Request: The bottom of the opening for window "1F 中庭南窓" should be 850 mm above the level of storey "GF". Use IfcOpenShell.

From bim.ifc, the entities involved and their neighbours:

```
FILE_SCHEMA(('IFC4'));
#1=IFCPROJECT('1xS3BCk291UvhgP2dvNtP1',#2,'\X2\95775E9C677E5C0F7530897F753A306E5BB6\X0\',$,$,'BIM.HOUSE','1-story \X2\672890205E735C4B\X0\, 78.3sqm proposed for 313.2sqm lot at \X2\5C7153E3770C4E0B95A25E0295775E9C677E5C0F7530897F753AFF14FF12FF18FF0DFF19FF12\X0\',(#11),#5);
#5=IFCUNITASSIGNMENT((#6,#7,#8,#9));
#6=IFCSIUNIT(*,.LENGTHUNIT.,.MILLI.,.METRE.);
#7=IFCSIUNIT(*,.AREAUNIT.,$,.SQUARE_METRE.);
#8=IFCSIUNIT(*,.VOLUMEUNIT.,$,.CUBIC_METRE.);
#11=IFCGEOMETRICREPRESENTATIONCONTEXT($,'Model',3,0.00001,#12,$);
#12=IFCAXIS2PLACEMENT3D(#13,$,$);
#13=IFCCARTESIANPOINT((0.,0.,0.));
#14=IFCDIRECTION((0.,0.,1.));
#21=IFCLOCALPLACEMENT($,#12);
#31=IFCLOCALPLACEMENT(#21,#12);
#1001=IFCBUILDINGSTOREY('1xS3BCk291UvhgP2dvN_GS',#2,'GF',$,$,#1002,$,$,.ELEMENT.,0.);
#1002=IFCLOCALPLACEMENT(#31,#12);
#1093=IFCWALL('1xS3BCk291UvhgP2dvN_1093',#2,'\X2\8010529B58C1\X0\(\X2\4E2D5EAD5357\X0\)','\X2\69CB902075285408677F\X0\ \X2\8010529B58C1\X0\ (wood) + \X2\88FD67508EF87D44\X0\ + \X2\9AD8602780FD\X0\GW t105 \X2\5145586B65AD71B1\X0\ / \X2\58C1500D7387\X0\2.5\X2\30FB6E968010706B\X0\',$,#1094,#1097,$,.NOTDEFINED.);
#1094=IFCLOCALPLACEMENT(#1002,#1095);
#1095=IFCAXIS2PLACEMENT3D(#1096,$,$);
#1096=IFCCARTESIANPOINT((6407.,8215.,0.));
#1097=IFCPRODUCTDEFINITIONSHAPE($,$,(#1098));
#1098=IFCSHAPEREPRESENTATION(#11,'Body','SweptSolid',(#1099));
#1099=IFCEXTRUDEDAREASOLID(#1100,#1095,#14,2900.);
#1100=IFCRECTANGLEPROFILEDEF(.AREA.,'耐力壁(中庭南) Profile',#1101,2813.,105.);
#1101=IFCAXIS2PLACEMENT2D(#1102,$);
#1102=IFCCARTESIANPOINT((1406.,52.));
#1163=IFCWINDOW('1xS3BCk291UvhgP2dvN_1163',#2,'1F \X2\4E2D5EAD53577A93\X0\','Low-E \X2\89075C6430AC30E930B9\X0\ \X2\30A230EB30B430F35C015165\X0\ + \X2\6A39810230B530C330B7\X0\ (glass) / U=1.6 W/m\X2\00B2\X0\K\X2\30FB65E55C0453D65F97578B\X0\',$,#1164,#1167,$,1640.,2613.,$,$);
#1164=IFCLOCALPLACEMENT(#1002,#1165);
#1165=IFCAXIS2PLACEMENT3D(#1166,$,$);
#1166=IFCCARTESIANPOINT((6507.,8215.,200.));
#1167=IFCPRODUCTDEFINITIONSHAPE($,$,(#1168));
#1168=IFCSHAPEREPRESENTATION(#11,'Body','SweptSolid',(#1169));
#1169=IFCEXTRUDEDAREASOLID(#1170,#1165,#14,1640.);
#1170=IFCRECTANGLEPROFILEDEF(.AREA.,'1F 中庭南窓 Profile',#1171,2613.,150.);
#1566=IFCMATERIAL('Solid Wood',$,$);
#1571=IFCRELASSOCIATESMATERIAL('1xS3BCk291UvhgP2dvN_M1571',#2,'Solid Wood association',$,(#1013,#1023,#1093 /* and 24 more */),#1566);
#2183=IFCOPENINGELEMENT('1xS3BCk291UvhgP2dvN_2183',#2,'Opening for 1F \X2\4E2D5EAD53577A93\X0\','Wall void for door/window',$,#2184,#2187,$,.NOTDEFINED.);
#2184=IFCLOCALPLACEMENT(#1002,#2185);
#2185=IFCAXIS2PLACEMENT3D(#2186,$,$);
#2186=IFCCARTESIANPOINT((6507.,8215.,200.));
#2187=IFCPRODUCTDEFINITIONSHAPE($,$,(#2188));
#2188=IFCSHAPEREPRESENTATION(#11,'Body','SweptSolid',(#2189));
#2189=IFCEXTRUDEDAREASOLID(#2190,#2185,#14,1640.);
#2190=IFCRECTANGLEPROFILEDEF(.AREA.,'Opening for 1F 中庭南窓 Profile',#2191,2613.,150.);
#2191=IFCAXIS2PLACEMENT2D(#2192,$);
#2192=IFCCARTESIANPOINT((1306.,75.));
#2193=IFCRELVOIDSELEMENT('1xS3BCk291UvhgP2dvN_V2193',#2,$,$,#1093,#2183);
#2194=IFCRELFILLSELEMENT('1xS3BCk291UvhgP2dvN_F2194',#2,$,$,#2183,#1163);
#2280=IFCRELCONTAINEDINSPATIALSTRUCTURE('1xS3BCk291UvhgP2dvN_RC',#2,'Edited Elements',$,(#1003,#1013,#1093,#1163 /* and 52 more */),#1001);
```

```python
import numpy as np
import ifcopenshell
import ifcopenshell.api.geometry
import ifcopenshell.geom
import ifcopenshell.util.element
import ifcopenshell.util.placement
import ifcopenshell.util.shape
import ifcopenshell.util.unit

model = ifcopenshell.open("bim.ifc")
unit_scale = ifcopenshell.util.unit.calculate_unit_scale(model)

window = model.by_guid("1xS3BCk291UvhgP2dvN_1163")
opening = window.FillsVoids[0].RelatingOpeningElement
storey = ifcopenshell.util.element.get_container(window, ifc_class="IfcBuildingStorey")
level = ifcopenshell.util.placement.get_local_placement(storey.ObjectPlacement)[2, 3]

# The opening's origin need not be at the sill, so measure its lowest point.
shape = ifcopenshell.geom.create_shape(ifcopenshell.geom.settings(), opening)
bottom = ifcopenshell.util.shape.get_shape_bottom_elevation(shape, shape.geometry) / unit_scale
dz = level + 0.85 / unit_scale - bottom

shift = np.array([0.0, 0.0, dz])
# The window is not placed relative to its opening, so move both.
for product in (opening, window):
    matrix = ifcopenshell.util.placement.get_local_placement(product.ObjectPlacement)
    matrix[:3, 3] += shift
    ifcopenshell.api.geometry.edit_object_placement(model, product=product, matrix=matrix, is_si=False)

print(f"moved by {dz * unit_scale:+.3f} m")

model.write("bim_updated.ifc")
```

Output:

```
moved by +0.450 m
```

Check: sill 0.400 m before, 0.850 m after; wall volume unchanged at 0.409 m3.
